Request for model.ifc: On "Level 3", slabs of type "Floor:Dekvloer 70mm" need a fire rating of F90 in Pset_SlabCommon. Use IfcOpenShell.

First a look at what the model holds.

```python
import ifcopenshell
import ifcopenshell.util.element

model = ifcopenshell.open("model.ifc")
print(model.schema)
storey = next(s for s in model.by_type("IfcBuildingStorey") if s.Name == "Level 3")
slabs = [e for e in ifcopenshell.util.element.get_decomposition(storey) if e.is_a("IfcSlab")]
seen = {}
for e in slabs:
    element_type = ifcopenshell.util.element.get_type(e)
    key = (element_type.Name if element_type != e and element_type else None, ifcopenshell.util.element.get_pset(e, "Pset_SlabCommon", "FireRating"))
    seen[key] = seen.get(key, 0) + 1
for (name, value), count in sorted(seen.items(), key=str):
    print(count, "x", name, "|", value)
```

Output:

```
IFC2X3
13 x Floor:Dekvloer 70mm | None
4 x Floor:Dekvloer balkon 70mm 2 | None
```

```python
import ifcopenshell
import ifcopenshell.api.pset
import ifcopenshell.util.element

model = ifcopenshell.open("model.ifc")

storey = next(s for s in model.by_type("IfcBuildingStorey") if s.Name == "Level 3")
slabs = [e for e in ifcopenshell.util.element.get_decomposition(storey) if e.is_a("IfcSlab")]

count = 0
for e in slabs:
    element_type = ifcopenshell.util.element.get_type(e)
    if element_type in (None, e) or element_type.Name != "Floor:Dekvloer 70mm":
        continue
    # add_pset returns the element's existing set when there is one.
    pset = ifcopenshell.api.pset.add_pset(model, product=e, name="Pset_SlabCommon")
    ifcopenshell.api.pset.edit_pset(model, pset=pset, properties={"FireRating": "F90"})
    count += 1

print(count, "slabs updated")

model.write("model_updated.ifc")
```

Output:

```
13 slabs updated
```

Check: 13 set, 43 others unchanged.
